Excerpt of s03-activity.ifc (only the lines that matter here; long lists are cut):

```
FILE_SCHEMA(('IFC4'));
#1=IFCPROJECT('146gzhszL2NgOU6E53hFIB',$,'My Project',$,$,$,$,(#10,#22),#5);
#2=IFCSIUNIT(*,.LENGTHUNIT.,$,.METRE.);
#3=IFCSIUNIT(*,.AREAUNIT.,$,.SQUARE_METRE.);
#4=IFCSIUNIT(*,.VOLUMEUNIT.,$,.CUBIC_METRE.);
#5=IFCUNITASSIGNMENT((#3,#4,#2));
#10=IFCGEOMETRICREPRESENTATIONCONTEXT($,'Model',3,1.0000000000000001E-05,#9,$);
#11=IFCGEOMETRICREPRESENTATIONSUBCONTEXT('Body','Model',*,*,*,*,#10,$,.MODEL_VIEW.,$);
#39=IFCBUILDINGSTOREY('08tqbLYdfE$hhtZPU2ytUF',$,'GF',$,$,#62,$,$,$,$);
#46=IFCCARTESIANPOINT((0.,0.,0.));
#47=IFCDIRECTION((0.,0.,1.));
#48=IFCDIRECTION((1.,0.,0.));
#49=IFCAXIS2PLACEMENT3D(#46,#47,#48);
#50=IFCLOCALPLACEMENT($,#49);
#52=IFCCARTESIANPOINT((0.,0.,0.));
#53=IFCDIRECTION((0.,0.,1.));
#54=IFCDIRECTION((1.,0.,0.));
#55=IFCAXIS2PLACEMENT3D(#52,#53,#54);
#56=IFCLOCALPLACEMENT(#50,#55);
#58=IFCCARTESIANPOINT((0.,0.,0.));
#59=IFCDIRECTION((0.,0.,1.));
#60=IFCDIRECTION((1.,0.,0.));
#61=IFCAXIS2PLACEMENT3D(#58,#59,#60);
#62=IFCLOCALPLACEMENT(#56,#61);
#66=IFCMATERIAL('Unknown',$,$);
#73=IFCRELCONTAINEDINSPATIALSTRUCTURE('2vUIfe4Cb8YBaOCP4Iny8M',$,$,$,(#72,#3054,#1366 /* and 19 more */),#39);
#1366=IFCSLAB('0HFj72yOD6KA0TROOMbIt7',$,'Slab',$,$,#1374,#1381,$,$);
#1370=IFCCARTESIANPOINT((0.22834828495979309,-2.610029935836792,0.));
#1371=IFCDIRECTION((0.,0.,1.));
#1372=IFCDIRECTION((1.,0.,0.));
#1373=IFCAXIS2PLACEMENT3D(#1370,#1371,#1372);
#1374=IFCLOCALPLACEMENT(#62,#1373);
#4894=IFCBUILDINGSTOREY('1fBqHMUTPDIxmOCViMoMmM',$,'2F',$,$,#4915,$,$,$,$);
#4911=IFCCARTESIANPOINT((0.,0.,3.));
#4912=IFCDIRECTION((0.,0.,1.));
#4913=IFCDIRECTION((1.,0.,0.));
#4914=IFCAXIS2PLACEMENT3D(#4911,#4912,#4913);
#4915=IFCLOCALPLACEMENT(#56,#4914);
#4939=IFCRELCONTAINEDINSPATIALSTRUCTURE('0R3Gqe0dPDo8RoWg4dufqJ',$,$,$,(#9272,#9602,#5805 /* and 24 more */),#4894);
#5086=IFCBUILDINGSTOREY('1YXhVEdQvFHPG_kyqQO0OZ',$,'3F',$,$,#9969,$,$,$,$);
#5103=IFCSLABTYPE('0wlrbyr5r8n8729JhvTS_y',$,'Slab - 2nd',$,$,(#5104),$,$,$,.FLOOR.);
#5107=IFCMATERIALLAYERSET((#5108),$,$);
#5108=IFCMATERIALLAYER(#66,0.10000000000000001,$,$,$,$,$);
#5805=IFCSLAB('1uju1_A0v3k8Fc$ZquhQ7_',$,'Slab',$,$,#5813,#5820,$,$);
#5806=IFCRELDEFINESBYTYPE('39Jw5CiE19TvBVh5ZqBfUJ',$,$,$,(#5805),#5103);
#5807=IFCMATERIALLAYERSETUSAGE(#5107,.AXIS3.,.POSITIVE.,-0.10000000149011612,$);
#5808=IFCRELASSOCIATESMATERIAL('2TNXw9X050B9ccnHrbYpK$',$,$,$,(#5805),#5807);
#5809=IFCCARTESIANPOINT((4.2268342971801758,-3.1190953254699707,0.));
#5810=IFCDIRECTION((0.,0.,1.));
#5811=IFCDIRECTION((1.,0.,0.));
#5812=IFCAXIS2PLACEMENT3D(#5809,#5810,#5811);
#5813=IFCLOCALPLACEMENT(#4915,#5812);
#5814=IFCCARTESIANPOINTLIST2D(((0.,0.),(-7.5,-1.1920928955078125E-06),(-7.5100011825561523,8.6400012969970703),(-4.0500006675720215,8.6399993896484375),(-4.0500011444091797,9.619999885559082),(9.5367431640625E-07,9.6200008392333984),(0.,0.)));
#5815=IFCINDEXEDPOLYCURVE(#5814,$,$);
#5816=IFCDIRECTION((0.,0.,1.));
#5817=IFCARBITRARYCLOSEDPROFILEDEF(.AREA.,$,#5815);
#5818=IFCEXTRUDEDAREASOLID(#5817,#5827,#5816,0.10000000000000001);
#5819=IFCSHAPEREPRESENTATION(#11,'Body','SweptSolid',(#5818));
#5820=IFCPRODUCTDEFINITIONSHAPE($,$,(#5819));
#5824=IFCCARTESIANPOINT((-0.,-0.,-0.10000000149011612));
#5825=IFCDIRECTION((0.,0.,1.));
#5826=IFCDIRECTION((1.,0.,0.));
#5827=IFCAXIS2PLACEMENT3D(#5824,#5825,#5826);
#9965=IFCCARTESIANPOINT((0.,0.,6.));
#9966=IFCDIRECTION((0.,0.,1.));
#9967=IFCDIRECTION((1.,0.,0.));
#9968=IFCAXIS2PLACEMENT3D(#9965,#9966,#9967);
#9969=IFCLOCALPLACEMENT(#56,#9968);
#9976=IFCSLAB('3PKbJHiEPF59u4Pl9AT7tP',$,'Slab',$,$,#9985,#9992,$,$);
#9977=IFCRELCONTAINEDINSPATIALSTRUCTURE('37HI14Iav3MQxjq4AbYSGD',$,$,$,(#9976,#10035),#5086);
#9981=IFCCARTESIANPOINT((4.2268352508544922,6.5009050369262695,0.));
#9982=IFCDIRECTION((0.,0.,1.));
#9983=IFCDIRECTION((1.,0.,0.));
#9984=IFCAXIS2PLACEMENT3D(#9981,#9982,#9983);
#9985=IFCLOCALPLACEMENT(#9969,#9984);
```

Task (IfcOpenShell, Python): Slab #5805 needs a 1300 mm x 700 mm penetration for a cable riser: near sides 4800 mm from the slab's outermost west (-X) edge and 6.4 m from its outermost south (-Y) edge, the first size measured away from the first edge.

```python
import numpy as np
import ifcopenshell
import ifcopenshell.api.feature
import ifcopenshell.api.geometry
import ifcopenshell.api.root
import ifcopenshell.geom
import ifcopenshell.util.placement
import ifcopenshell.util.representation
import ifcopenshell.util.shape
import ifcopenshell.util.unit

model = ifcopenshell.open("s03-activity.ifc")
unit_scale = ifcopenshell.util.unit.calculate_unit_scale(model)
settings = ifcopenshell.geom.settings()


def volume(element):
    """Net volume in cubic metres, openings subtracted."""
    shape = ifcopenshell.geom.create_shape(settings, element)
    return ifcopenshell.util.shape.get_volume(shape.geometry)


slab = model.by_id(5805)
before = volume(slab)

# Extent in the slab's own axes, in metres. The edges named are its -X and -Y sides.
slab_shape = ifcopenshell.geom.create_shape(settings, slab)
vertices = ifcopenshell.util.shape.get_vertices(slab_shape.geometry)
x_min, y_min, bottom = vertices.min(axis=0)
top = vertices[:, 2].max()

opening = ifcopenshell.api.root.create_entity(model, ifc_class="IfcOpeningElement", name="Cable riser opening", predefined_type="OPENING")
context = ifcopenshell.util.representation.get_context(model, "Model", "Body", "MODEL_VIEW")
width, depth = 1.3, 0.7
outline = [(0.0, 0.0), (width, 0.0), (width, depth), (0.0, depth), (0.0, 0.0)]
# Overshoot both faces by 50 mm so the cut is clean.
shape = ifcopenshell.api.geometry.add_slab_representation(
    model, context=context, depth=top - bottom + 0.1, polyline=outline
)
ifcopenshell.api.geometry.assign_representation(model, product=opening, representation=shape)

matrix = ifcopenshell.util.placement.get_local_placement(slab.ObjectPlacement)
matrix[:, 3] = matrix @ np.append(np.array([x_min + 4.8, y_min + 6.4, bottom - 0.05]) / unit_scale, 1.0)
ifcopenshell.api.geometry.edit_object_placement(model, product=opening, matrix=matrix, is_si=False)
ifcopenshell.api.feature.add_feature(model, feature=opening, element=slab)

after = volume(slab)

print(f"slab volume {before:.3f} -> {after:.3f} m3")

model.write("s03-activity_updated.ifc")
```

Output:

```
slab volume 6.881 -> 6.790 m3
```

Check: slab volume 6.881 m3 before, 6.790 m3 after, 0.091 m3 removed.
